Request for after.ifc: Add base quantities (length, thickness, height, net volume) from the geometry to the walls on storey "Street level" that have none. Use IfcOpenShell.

First a look at what the model holds.

```python
import ifcopenshell
import ifcopenshell.util.element
import ifcopenshell.util.unit

model = ifcopenshell.open("after.ifc")
print(model.schema)
for unit_type in ("LENGTHUNIT", "AREAUNIT", "VOLUMEUNIT"):
    print(unit_type, ifcopenshell.util.unit.calculate_unit_scale(model, unit_type))
storey = next(s for s in model.by_type("IfcBuildingStorey") if s.Name == "Street level")
walls = [e for e in ifcopenshell.util.element.get_decomposition(storey) if e.is_a("IfcWall")]
for e in sorted(walls, key=lambda e: e.id()):
    print(e.id(), e.is_a(), e.Name, list(ifcopenshell.util.element.get_psets(e, qtos_only=True)), sep=" | ")
```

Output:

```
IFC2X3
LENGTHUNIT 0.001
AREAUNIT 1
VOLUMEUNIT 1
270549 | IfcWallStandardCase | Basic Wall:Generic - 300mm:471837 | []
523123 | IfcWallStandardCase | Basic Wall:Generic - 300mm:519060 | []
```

```python
import ifcopenshell
import ifcopenshell.api.pset
import ifcopenshell.geom
import ifcopenshell.util.element
import ifcopenshell.util.shape
import ifcopenshell.util.unit

model = ifcopenshell.open("after.ifc")
unit_scale = ifcopenshell.util.unit.calculate_unit_scale(model)
volume_scale = ifcopenshell.util.unit.calculate_unit_scale(model, "VOLUMEUNIT")
settings = ifcopenshell.geom.settings()

storey = next(s for s in model.by_type("IfcBuildingStorey") if s.Name == "Street level")
walls = [e for e in ifcopenshell.util.element.get_decomposition(storey) if e.is_a("IfcWall")]

for e in sorted(walls, key=lambda e: e.id()):
    if ifcopenshell.util.element.get_psets(e, qtos_only=True, should_inherit=False):
        continue
    # Geometry comes back in metres, in the element's own axes.
    shape = ifcopenshell.geom.create_shape(settings, e)
    values = {
        "Length": ifcopenshell.util.shape.get_x(shape.geometry) / unit_scale,
        "Width": ifcopenshell.util.shape.get_y(shape.geometry) / unit_scale,
        "Height": ifcopenshell.util.shape.get_z(shape.geometry) / unit_scale,
        "NetVolume": ifcopenshell.util.shape.get_volume(shape.geometry) / volume_scale,
    }
    qto = ifcopenshell.api.pset.add_qto(model, product=e, name="BaseQuantities")
    ifcopenshell.api.pset.edit_qto(model, qto=qto, properties=values)
    print(e.id(), {k: round(v, 3) for k, v in values.items()})

model.write("after_updated.ifc")
```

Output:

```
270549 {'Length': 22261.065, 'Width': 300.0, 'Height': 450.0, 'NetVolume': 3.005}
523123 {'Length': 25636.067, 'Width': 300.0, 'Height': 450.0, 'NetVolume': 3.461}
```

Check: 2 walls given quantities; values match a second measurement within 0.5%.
